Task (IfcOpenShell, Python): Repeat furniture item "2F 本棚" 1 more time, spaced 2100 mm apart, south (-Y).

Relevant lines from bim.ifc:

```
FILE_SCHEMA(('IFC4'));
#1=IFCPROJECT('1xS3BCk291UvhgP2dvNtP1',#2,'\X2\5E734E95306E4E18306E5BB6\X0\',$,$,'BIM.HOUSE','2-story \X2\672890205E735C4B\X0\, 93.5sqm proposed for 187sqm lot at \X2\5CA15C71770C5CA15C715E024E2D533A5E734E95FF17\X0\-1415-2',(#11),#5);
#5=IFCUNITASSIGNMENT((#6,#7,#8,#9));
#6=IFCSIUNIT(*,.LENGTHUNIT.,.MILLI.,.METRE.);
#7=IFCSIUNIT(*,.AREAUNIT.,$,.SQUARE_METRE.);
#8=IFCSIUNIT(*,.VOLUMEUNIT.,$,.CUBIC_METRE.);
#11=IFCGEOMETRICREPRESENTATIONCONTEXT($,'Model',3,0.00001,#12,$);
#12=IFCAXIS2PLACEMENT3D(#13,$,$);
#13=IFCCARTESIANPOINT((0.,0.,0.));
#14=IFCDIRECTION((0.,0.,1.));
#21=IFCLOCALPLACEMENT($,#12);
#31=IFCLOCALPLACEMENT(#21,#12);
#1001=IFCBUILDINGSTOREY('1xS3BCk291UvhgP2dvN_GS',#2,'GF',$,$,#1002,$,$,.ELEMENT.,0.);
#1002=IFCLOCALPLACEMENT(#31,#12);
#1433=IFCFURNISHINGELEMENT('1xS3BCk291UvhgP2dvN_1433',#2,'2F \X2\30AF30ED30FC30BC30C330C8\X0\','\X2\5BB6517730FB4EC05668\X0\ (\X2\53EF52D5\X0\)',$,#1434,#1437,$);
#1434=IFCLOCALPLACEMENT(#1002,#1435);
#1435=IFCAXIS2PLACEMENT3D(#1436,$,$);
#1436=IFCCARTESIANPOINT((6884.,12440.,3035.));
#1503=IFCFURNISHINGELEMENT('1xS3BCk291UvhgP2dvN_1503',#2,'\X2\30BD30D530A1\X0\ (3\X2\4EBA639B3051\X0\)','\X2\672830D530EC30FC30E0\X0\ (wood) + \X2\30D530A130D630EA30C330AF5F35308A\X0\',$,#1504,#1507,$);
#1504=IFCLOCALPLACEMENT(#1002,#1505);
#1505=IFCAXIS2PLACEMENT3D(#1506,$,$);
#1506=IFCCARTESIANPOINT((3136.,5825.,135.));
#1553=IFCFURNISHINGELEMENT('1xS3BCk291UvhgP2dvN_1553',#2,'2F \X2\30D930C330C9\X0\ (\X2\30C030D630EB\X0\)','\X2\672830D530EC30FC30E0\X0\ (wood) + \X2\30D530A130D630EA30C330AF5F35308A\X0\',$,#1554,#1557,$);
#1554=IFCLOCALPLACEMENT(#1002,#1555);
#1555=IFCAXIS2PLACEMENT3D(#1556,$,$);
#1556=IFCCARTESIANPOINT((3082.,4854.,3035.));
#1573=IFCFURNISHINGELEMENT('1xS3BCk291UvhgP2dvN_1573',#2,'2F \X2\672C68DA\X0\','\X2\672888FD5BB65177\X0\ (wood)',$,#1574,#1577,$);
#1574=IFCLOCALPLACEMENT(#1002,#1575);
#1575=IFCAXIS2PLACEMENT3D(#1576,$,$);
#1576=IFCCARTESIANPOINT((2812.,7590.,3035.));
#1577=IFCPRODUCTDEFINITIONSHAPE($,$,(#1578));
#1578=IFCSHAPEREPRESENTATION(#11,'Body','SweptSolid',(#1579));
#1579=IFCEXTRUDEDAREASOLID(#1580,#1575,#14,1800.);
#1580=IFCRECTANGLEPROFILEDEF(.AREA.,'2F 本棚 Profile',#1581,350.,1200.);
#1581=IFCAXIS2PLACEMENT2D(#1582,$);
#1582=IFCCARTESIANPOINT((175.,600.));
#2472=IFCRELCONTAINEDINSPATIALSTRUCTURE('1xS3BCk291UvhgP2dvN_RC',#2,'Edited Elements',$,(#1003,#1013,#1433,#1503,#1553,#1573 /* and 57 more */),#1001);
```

```python
import numpy as np
import ifcopenshell
import ifcopenshell.api.geometry
import ifcopenshell.api.root
import ifcopenshell.util.element
import ifcopenshell.util.placement
import ifcopenshell.util.unit

model = ifcopenshell.open("bim.ifc")
unit_scale = ifcopenshell.util.unit.calculate_unit_scale(model)


def reuse_history(source, copy):
    """copy_class also copies each property set's owner history, people and application; keep the originals."""
    for rel in copy.IsDefinedBy:
        if rel.is_a("IfcRelDefinesByProperties") and (history := rel.RelatingPropertyDefinition.OwnerHistory):
            rel.RelatingPropertyDefinition.OwnerHistory = source.OwnerHistory
            ifcopenshell.util.element.remove_deep2(model, history)


source = model.by_guid("1xS3BCk291UvhgP2dvN_1573")
base = ifcopenshell.util.placement.get_local_placement(source.ObjectPlacement)
step = np.array([0.0, -1.0, 0.0]) * 2.1 / unit_scale

for i in range(1, 2):
    copy = ifcopenshell.api.root.copy_class(model, product=source)
    copy.Representation = ifcopenshell.util.element.copy_deep(
        model, source.Representation, exclude=["IfcGeometricRepresentationContext", "IfcRepresentationMap"]
    )
    reuse_history(source, copy)
    matrix = base.copy()
    matrix[:3, 3] += i * step
    print("added at", matrix[:3, 3].round(3) + 0.0)
    ifcopenshell.api.geometry.edit_object_placement(model, product=copy, matrix=matrix, is_si=False)

model.write("bim_updated.ifc")
```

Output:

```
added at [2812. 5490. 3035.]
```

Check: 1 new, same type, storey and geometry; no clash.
